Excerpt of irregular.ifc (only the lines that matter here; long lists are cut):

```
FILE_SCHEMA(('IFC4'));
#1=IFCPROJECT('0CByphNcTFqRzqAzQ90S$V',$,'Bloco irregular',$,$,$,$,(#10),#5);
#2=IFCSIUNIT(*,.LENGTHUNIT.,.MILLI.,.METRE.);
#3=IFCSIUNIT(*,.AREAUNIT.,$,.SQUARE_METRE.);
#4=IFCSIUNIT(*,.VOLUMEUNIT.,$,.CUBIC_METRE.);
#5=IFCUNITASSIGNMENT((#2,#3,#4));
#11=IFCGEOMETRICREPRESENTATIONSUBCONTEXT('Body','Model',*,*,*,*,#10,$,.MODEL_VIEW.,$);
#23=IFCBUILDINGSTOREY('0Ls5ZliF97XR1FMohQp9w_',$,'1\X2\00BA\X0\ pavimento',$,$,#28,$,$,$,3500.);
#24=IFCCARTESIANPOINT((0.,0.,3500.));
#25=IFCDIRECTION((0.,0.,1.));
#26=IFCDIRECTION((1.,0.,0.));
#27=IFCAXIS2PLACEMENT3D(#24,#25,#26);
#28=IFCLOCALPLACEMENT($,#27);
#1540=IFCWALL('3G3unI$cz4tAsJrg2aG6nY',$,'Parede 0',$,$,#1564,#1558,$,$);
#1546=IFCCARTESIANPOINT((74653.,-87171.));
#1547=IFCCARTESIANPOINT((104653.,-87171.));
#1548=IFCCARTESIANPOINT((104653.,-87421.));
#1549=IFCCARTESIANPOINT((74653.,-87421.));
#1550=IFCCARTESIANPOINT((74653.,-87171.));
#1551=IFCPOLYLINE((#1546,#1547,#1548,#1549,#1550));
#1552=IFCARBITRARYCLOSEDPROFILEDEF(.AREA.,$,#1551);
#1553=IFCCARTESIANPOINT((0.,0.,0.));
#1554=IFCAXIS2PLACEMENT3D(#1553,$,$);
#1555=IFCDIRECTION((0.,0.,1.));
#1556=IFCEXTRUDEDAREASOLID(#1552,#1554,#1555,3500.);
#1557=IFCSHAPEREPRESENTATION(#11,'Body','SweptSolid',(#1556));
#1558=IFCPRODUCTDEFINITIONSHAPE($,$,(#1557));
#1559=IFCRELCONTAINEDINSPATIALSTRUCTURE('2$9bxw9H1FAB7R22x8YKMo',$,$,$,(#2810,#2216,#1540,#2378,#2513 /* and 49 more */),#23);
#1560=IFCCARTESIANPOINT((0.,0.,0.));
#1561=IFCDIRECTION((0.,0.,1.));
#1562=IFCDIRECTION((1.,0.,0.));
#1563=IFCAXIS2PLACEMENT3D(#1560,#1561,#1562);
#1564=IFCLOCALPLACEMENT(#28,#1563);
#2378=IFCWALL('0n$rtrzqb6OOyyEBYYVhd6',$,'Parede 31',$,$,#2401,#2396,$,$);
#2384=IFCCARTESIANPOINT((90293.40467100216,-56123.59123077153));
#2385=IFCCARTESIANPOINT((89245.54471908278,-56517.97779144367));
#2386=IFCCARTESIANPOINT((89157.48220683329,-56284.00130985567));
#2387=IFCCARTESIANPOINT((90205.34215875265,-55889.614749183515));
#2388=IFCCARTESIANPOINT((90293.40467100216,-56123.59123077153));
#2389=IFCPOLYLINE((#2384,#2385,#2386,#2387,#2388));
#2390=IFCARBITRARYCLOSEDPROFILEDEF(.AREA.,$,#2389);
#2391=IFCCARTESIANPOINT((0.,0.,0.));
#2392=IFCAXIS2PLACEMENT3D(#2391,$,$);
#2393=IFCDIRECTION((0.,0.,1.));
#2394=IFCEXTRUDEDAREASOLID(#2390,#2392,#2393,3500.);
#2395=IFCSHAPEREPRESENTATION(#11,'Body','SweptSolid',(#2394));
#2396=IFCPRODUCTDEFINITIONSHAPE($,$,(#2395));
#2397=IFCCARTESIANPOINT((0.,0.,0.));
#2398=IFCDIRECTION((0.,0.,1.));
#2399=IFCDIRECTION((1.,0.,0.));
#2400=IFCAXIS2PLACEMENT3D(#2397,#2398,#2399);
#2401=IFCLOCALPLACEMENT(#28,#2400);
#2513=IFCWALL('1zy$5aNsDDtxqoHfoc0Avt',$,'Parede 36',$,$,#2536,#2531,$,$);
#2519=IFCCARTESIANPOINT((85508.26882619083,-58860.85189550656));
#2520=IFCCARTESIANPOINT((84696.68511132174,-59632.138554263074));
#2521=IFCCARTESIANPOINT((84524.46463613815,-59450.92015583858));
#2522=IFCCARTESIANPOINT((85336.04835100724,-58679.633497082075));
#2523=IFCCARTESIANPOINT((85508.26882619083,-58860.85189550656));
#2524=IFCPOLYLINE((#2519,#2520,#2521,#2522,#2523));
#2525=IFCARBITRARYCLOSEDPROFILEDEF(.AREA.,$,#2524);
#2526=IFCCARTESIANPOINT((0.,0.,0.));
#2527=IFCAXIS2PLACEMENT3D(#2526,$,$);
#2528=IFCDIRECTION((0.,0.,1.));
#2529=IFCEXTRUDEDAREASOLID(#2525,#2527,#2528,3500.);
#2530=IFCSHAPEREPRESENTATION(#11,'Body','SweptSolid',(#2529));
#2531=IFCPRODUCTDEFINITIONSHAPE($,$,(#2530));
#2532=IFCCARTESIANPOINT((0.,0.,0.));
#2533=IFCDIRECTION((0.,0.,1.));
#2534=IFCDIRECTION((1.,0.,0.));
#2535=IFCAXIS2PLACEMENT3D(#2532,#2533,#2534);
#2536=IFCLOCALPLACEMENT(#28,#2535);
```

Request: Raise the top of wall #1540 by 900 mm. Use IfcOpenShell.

```python
import ifcopenshell
import ifcopenshell.geom
import ifcopenshell.util.representation
import ifcopenshell.util.shape

model = ifcopenshell.open("irregular.ifc")
settings = ifcopenshell.geom.settings()


def volume(element):
    """Net volume in cubic metres, openings subtracted."""
    shape = ifcopenshell.geom.create_shape(settings, element)
    return ifcopenshell.util.shape.get_volume(shape.geometry)


wall = model.by_guid("3G3unI$cz4tAsJrg2aG6nY")
before = volume(wall)

body = ifcopenshell.util.representation.get_representation(wall, "Model", "Body")
solid = body.Items[0]
old_height = solid.Depth
solid.Depth += 900.0
after = volume(wall)

print(f"height {old_height:g} -> {solid.Depth:g}, volume {before:.3f} -> {after:.3f} m3")

model.write("irregular-out.ifc")
```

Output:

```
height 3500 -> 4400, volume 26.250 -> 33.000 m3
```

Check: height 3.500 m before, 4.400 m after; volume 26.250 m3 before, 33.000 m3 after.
